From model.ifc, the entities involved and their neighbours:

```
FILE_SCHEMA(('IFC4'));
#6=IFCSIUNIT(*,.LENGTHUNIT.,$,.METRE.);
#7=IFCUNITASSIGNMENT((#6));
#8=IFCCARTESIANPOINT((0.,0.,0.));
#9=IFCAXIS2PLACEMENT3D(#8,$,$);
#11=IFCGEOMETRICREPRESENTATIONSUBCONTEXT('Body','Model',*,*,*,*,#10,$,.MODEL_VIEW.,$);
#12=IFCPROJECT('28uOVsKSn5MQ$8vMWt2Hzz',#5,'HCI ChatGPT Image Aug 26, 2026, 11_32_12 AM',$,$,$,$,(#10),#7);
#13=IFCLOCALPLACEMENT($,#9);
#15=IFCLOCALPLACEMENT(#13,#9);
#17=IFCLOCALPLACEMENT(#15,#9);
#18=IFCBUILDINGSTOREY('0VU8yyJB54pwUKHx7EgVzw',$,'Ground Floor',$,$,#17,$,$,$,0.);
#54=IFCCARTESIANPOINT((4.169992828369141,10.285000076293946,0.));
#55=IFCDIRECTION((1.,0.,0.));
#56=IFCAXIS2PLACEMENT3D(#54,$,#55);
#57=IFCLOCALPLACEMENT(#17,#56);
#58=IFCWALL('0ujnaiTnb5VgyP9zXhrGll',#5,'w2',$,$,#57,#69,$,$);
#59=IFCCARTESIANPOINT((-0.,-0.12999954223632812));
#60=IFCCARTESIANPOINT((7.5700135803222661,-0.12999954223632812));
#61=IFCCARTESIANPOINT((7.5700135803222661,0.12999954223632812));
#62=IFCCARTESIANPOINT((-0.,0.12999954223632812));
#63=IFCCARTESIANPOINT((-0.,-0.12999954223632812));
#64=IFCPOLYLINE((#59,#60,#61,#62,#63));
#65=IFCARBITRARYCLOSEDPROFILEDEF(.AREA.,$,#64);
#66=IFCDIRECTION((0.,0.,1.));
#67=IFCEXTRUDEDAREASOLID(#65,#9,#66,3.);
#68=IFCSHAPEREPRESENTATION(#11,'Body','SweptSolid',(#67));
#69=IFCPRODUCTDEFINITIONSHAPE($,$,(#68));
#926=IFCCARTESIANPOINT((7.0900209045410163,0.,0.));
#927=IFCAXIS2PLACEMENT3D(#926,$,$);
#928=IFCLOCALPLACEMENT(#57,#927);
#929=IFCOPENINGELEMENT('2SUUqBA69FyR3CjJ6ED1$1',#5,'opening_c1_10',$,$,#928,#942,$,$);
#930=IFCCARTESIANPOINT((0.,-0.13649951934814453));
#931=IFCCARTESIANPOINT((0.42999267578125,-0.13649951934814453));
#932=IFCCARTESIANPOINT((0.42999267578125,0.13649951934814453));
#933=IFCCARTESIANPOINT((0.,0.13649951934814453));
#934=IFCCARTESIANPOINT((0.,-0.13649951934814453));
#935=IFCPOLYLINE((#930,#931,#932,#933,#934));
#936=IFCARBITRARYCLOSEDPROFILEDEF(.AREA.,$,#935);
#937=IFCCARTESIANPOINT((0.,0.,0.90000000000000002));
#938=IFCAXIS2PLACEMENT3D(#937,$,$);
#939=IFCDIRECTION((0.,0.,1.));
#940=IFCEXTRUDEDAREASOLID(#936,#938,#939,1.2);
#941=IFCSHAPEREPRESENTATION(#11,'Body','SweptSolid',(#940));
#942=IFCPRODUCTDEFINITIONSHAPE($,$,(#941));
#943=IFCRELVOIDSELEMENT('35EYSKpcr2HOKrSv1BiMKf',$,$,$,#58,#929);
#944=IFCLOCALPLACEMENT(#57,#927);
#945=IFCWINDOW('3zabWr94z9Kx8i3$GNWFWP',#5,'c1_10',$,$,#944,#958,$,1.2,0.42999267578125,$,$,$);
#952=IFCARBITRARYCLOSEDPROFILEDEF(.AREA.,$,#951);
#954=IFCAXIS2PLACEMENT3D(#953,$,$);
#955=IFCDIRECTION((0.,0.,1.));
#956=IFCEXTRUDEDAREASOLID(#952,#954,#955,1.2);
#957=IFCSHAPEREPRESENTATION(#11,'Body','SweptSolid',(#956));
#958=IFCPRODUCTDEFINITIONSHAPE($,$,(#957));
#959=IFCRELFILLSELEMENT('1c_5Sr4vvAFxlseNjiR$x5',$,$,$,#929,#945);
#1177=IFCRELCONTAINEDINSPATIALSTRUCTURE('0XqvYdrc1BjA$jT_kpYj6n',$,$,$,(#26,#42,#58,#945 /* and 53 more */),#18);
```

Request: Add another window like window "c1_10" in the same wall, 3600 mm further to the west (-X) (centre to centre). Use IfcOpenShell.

```python
import ifcopenshell
import ifcopenshell.api.feature
import ifcopenshell.api.geometry
import ifcopenshell.api.root
import ifcopenshell.geom
import ifcopenshell.util.element
import ifcopenshell.util.placement
import ifcopenshell.util.shape

model = ifcopenshell.open("model.ifc")
settings = ifcopenshell.geom.settings()


def volume(element):
    """Net volume in cubic metres, openings subtracted."""
    shape = ifcopenshell.geom.create_shape(settings, element)
    return ifcopenshell.util.shape.get_volume(shape.geometry)


window = model.by_id(945)
opening = window.FillsVoids[0].RelatingOpeningElement
wall = opening.VoidsElements[0].RelatingBuildingElement
before = volume(wall)
shift = ifcopenshell.util.placement.get_local_placement(wall.ObjectPlacement)[:3, 0] * -3.6

# copy_class copies the void relationship, type, container and properties, but no geometry.
new_opening = ifcopenshell.api.root.copy_class(model, product=opening)
new_opening.Representation = ifcopenshell.util.element.copy_deep(
    model, opening.Representation, exclude=["IfcGeometricRepresentationContext", "IfcRepresentationMap"]
)
new_window = ifcopenshell.api.root.copy_class(model, product=window)
new_window.Representation = ifcopenshell.util.element.copy_deep(
    model, window.Representation, exclude=["IfcGeometricRepresentationContext", "IfcRepresentationMap"]
)
ifcopenshell.api.feature.add_filling(model, opening=new_opening, element=new_window)

for old, new in ((opening, new_opening), (window, new_window)):
    matrix = ifcopenshell.util.placement.get_local_placement(old.ObjectPlacement)
    matrix[:3, 3] += shift
    ifcopenshell.api.geometry.edit_object_placement(model, product=new, matrix=matrix, is_si=False)

after = volume(wall)

print(f"wall volume {before:.3f} -> {after:.3f} m3")

model.write("model_rev.ifc")
```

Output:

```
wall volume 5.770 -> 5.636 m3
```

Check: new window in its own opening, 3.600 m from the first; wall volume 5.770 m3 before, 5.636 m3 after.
